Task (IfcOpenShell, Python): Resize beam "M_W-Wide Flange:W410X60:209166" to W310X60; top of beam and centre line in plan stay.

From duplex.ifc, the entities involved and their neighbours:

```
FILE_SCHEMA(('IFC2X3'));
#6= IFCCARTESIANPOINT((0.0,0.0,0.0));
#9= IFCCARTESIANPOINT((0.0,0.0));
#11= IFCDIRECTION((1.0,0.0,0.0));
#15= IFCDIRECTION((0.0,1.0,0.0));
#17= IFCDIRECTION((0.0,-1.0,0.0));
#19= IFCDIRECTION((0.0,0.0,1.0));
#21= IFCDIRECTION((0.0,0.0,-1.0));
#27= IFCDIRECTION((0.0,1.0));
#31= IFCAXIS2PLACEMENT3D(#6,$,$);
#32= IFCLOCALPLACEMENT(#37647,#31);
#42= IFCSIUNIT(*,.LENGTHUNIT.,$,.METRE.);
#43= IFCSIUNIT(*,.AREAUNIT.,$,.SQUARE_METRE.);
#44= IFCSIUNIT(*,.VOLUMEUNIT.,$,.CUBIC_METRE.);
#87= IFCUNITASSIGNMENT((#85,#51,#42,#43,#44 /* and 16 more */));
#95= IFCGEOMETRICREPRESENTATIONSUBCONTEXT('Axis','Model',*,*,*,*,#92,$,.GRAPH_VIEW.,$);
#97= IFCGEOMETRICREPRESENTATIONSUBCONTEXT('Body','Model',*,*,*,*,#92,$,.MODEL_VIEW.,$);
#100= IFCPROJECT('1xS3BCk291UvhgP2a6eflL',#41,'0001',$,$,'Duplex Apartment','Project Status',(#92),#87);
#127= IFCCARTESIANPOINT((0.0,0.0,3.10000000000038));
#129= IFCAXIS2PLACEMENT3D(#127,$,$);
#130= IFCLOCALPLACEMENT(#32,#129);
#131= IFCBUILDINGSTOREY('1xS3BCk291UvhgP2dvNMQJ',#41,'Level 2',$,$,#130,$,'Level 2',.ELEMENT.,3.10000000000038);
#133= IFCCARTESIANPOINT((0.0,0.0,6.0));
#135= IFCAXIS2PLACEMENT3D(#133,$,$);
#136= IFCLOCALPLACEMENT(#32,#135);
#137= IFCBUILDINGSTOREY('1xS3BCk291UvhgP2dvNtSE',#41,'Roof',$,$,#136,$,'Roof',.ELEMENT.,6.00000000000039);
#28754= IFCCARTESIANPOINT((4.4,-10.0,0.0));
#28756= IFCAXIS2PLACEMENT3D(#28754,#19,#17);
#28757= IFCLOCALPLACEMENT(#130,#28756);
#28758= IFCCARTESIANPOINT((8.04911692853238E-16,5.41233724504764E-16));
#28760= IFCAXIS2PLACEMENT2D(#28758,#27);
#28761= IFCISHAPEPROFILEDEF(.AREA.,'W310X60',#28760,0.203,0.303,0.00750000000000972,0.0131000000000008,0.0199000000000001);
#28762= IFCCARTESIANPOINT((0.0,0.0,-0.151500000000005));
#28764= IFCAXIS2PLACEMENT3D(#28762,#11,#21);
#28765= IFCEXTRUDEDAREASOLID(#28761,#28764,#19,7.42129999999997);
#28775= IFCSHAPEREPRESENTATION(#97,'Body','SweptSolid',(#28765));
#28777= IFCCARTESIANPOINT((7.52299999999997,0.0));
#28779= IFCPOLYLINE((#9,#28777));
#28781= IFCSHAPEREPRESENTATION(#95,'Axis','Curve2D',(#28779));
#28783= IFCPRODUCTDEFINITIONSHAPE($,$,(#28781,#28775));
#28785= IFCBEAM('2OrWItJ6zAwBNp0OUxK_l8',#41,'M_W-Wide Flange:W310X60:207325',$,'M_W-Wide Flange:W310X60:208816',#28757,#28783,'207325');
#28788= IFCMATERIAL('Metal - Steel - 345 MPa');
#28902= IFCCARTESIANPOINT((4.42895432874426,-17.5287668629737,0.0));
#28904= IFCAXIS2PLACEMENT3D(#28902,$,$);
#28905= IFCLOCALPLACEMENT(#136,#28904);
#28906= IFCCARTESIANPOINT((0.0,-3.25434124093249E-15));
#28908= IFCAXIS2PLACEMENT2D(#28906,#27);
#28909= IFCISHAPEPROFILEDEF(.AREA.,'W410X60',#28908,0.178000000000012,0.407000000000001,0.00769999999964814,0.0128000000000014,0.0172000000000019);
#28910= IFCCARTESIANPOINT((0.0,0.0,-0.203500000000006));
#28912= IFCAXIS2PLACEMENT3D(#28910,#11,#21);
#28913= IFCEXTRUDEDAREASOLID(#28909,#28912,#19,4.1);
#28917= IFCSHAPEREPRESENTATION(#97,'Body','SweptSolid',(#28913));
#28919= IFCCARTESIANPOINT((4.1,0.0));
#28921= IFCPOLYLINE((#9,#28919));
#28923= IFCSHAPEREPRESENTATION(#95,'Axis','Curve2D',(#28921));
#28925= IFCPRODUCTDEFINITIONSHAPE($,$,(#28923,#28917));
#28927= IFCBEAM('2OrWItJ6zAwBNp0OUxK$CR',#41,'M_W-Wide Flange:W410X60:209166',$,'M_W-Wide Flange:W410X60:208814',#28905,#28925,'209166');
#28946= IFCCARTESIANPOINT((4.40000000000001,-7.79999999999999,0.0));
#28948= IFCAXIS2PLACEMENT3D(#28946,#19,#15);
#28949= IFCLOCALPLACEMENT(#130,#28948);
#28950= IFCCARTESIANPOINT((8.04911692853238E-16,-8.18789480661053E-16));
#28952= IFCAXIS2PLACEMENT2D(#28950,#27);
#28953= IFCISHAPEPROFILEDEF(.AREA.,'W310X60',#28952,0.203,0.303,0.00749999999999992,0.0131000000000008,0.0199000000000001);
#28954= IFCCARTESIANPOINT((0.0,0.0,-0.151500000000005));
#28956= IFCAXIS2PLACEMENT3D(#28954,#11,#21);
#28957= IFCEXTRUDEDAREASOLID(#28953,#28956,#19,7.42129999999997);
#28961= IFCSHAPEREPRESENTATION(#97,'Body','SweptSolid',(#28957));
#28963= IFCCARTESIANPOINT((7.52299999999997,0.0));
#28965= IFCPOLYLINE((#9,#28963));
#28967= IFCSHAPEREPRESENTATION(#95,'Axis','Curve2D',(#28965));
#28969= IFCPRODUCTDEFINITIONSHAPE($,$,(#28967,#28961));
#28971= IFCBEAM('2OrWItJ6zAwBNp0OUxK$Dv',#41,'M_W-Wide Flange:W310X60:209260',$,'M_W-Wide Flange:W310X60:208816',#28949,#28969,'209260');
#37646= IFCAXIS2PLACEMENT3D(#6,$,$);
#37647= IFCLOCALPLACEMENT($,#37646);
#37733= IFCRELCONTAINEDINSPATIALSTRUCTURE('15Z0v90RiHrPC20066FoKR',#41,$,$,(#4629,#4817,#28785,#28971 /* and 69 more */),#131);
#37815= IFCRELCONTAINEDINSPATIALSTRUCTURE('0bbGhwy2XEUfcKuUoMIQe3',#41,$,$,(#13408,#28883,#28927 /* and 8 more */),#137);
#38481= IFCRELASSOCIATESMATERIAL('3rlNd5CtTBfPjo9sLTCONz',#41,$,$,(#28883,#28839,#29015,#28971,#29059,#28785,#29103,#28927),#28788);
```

```python
import ifcopenshell
import ifcopenshell.util.element
import ifcopenshell.util.representation

model = ifcopenshell.open("duplex.ifc")

member = model.by_guid("2OrWItJ6zAwBNp0OUxK$CR")
source = next(p for p in model.by_type("IfcIShapeProfileDef") if p.ProfileName == "W310X60")

body = ifcopenshell.util.representation.get_representation(member, "Model", "Body")
solid = body.Items[0]
old_profile = solid.SweptArea

# Copy the section's sizes but keep this member's own profile position.
profile = ifcopenshell.util.element.copy(model, source)
# Profiles are centred, so shift by half the change in depth to hold the top.
shift = (old_profile.OverallDepth - profile.OverallDepth) / 2
x, y = old_profile.Position.Location.Coordinates
up = (-1.0, 0.0)  # upwards, in the solid's own plane
location = model.createIfcCartesianPoint((x + up[0] * shift, y + up[1] * shift))
profile.Position = model.createIfcAxis2Placement2D(location, old_profile.Position.RefDirection)
solid.SweptArea = profile
if not model.get_total_inverses(old_profile):
    ifcopenshell.util.element.remove_deep2(model, old_profile)
member.Name = member.Name.replace("W410X60", "W310X60")
member.ObjectType = member.ObjectType.replace("W410X60", "W310X60")

print(solid.SweptArea)

model.write("duplex_edited.ifc")
```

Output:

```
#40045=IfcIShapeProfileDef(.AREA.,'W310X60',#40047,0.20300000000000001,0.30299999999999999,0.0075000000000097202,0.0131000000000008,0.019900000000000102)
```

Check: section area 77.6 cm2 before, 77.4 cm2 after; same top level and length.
